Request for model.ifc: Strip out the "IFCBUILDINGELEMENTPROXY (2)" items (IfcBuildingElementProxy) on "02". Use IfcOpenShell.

First a look at what the model holds.

```python
import ifcopenshell
import ifcopenshell.util.element

model = ifcopenshell.open("model.ifc")
print(model.schema)
storey = next(s for s in model.by_type("IfcBuildingStorey") if s.Name == "02")
proxies = [e for e in ifcopenshell.util.element.get_decomposition(storey) if e.is_a("IfcBuildingElementProxy")]
seen = {}
for e in proxies:
    element_type = ifcopenshell.util.element.get_type(e)
    name = element_type.Name if element_type not in (None, e) else None
    seen[name] = seen.get(name, 0) + 1
for name, count in sorted(seen.items(), key=str):
    print(count, "x", name)
```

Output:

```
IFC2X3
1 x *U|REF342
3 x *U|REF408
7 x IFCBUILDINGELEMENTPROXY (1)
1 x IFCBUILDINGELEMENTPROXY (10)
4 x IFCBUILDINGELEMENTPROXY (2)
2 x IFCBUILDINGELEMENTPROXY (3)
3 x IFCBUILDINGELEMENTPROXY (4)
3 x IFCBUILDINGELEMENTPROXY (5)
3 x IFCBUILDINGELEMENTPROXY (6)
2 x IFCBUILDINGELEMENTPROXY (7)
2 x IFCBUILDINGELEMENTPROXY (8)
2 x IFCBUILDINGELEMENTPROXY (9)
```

```python
import ifcopenshell
import ifcopenshell.api.root
import ifcopenshell.util.element

model = ifcopenshell.open("model.ifc")

storey = next(s for s in model.by_type("IfcBuildingStorey") if s.Name == "02")
proxies = [e for e in ifcopenshell.util.element.get_decomposition(storey) if e.is_a("IfcBuildingElementProxy")]
targets = [e for e in proxies if (t := ifcopenshell.util.element.get_type(e)) not in (None, e) and t.Name == "IFCBUILDINGELEMENTPROXY (2)"]

for e in targets:
    ifcopenshell.api.root.remove_product(model, product=e)
print(len(targets), "removed")

model.write("model_rev.ifc")
```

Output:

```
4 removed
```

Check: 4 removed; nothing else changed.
